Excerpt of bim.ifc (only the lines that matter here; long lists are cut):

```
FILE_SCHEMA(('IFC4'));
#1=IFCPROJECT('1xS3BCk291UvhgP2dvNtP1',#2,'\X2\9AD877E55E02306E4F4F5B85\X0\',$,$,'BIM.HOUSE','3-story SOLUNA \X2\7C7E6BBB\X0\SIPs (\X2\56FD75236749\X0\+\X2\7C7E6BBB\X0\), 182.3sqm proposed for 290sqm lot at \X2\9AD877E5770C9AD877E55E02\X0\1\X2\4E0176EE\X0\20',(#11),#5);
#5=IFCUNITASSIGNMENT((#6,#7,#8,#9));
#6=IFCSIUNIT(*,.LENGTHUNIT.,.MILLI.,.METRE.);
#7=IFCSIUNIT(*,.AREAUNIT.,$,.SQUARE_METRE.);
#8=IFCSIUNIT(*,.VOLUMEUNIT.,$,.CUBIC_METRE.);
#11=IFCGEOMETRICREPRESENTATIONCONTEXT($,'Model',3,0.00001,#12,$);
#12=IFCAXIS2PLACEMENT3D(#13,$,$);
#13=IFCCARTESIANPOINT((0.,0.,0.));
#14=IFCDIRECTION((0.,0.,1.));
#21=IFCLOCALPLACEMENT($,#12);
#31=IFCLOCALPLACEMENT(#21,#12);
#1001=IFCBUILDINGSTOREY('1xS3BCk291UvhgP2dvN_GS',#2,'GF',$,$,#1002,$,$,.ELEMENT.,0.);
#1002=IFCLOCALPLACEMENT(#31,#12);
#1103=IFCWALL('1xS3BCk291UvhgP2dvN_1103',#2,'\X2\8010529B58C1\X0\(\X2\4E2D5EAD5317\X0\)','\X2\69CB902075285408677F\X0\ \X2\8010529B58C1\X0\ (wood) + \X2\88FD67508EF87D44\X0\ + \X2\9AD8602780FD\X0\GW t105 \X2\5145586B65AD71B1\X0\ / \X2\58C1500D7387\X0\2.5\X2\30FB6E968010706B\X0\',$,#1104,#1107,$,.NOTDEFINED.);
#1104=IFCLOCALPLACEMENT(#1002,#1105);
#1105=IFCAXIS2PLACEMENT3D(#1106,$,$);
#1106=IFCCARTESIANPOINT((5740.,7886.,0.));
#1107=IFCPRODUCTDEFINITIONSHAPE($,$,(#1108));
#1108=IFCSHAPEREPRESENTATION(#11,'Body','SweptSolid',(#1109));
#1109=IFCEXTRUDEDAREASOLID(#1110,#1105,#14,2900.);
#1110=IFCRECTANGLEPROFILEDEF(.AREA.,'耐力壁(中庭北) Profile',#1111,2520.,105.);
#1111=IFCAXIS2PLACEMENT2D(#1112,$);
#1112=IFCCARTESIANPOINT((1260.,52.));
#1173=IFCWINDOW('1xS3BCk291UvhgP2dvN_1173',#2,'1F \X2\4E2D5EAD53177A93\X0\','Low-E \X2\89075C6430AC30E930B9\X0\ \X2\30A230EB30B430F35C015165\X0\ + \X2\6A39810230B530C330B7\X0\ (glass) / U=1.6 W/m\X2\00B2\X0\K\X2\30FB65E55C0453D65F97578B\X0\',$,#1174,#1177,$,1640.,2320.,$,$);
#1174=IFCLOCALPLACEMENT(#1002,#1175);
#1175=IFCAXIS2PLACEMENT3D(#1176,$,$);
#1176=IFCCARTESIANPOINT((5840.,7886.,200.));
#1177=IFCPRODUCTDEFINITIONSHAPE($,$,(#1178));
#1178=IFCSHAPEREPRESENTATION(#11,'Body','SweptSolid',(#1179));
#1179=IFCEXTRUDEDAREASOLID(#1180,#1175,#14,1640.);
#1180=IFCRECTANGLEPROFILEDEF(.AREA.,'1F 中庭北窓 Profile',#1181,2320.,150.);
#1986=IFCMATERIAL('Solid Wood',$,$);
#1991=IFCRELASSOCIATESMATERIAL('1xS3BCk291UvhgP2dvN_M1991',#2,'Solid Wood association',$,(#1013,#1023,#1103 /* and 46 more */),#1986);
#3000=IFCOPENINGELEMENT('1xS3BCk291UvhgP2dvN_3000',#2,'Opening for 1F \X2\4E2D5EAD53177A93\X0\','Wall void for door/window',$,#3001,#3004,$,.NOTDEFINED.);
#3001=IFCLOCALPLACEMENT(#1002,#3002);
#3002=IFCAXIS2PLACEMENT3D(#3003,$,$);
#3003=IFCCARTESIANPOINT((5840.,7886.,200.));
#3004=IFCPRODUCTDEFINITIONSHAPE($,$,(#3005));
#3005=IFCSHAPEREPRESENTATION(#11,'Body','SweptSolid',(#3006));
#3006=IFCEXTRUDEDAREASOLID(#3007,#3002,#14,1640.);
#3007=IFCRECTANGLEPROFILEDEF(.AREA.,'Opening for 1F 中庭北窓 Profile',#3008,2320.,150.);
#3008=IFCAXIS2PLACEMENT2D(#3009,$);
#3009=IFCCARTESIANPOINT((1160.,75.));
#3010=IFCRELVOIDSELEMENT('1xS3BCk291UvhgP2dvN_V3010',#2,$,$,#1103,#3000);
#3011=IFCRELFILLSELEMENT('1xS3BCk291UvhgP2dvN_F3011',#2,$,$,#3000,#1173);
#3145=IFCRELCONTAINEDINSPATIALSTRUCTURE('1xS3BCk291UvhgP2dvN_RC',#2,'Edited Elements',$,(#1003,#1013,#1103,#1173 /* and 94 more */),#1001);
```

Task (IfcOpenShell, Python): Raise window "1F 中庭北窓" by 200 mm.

```python
import numpy as np
import ifcopenshell
import ifcopenshell.api.geometry
import ifcopenshell.util.placement
import ifcopenshell.util.unit

model = ifcopenshell.open("bim.ifc")
unit_scale = ifcopenshell.util.unit.calculate_unit_scale(model)

window = model.by_guid("1xS3BCk291UvhgP2dvN_1173")
opening = window.FillsVoids[0].RelatingOpeningElement
dz = 200.0

shift = np.array([0.0, 0.0, dz])
# The window is not placed relative to its opening, so move both.
for product in (opening, window):
    matrix = ifcopenshell.util.placement.get_local_placement(product.ObjectPlacement)
    matrix[:3, 3] += shift
    ifcopenshell.api.geometry.edit_object_placement(model, product=product, matrix=matrix, is_si=False)

print(f"moved by {dz * unit_scale:+.3f} m")

model.write("bim-out.ifc")
```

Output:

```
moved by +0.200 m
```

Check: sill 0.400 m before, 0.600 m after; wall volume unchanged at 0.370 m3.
